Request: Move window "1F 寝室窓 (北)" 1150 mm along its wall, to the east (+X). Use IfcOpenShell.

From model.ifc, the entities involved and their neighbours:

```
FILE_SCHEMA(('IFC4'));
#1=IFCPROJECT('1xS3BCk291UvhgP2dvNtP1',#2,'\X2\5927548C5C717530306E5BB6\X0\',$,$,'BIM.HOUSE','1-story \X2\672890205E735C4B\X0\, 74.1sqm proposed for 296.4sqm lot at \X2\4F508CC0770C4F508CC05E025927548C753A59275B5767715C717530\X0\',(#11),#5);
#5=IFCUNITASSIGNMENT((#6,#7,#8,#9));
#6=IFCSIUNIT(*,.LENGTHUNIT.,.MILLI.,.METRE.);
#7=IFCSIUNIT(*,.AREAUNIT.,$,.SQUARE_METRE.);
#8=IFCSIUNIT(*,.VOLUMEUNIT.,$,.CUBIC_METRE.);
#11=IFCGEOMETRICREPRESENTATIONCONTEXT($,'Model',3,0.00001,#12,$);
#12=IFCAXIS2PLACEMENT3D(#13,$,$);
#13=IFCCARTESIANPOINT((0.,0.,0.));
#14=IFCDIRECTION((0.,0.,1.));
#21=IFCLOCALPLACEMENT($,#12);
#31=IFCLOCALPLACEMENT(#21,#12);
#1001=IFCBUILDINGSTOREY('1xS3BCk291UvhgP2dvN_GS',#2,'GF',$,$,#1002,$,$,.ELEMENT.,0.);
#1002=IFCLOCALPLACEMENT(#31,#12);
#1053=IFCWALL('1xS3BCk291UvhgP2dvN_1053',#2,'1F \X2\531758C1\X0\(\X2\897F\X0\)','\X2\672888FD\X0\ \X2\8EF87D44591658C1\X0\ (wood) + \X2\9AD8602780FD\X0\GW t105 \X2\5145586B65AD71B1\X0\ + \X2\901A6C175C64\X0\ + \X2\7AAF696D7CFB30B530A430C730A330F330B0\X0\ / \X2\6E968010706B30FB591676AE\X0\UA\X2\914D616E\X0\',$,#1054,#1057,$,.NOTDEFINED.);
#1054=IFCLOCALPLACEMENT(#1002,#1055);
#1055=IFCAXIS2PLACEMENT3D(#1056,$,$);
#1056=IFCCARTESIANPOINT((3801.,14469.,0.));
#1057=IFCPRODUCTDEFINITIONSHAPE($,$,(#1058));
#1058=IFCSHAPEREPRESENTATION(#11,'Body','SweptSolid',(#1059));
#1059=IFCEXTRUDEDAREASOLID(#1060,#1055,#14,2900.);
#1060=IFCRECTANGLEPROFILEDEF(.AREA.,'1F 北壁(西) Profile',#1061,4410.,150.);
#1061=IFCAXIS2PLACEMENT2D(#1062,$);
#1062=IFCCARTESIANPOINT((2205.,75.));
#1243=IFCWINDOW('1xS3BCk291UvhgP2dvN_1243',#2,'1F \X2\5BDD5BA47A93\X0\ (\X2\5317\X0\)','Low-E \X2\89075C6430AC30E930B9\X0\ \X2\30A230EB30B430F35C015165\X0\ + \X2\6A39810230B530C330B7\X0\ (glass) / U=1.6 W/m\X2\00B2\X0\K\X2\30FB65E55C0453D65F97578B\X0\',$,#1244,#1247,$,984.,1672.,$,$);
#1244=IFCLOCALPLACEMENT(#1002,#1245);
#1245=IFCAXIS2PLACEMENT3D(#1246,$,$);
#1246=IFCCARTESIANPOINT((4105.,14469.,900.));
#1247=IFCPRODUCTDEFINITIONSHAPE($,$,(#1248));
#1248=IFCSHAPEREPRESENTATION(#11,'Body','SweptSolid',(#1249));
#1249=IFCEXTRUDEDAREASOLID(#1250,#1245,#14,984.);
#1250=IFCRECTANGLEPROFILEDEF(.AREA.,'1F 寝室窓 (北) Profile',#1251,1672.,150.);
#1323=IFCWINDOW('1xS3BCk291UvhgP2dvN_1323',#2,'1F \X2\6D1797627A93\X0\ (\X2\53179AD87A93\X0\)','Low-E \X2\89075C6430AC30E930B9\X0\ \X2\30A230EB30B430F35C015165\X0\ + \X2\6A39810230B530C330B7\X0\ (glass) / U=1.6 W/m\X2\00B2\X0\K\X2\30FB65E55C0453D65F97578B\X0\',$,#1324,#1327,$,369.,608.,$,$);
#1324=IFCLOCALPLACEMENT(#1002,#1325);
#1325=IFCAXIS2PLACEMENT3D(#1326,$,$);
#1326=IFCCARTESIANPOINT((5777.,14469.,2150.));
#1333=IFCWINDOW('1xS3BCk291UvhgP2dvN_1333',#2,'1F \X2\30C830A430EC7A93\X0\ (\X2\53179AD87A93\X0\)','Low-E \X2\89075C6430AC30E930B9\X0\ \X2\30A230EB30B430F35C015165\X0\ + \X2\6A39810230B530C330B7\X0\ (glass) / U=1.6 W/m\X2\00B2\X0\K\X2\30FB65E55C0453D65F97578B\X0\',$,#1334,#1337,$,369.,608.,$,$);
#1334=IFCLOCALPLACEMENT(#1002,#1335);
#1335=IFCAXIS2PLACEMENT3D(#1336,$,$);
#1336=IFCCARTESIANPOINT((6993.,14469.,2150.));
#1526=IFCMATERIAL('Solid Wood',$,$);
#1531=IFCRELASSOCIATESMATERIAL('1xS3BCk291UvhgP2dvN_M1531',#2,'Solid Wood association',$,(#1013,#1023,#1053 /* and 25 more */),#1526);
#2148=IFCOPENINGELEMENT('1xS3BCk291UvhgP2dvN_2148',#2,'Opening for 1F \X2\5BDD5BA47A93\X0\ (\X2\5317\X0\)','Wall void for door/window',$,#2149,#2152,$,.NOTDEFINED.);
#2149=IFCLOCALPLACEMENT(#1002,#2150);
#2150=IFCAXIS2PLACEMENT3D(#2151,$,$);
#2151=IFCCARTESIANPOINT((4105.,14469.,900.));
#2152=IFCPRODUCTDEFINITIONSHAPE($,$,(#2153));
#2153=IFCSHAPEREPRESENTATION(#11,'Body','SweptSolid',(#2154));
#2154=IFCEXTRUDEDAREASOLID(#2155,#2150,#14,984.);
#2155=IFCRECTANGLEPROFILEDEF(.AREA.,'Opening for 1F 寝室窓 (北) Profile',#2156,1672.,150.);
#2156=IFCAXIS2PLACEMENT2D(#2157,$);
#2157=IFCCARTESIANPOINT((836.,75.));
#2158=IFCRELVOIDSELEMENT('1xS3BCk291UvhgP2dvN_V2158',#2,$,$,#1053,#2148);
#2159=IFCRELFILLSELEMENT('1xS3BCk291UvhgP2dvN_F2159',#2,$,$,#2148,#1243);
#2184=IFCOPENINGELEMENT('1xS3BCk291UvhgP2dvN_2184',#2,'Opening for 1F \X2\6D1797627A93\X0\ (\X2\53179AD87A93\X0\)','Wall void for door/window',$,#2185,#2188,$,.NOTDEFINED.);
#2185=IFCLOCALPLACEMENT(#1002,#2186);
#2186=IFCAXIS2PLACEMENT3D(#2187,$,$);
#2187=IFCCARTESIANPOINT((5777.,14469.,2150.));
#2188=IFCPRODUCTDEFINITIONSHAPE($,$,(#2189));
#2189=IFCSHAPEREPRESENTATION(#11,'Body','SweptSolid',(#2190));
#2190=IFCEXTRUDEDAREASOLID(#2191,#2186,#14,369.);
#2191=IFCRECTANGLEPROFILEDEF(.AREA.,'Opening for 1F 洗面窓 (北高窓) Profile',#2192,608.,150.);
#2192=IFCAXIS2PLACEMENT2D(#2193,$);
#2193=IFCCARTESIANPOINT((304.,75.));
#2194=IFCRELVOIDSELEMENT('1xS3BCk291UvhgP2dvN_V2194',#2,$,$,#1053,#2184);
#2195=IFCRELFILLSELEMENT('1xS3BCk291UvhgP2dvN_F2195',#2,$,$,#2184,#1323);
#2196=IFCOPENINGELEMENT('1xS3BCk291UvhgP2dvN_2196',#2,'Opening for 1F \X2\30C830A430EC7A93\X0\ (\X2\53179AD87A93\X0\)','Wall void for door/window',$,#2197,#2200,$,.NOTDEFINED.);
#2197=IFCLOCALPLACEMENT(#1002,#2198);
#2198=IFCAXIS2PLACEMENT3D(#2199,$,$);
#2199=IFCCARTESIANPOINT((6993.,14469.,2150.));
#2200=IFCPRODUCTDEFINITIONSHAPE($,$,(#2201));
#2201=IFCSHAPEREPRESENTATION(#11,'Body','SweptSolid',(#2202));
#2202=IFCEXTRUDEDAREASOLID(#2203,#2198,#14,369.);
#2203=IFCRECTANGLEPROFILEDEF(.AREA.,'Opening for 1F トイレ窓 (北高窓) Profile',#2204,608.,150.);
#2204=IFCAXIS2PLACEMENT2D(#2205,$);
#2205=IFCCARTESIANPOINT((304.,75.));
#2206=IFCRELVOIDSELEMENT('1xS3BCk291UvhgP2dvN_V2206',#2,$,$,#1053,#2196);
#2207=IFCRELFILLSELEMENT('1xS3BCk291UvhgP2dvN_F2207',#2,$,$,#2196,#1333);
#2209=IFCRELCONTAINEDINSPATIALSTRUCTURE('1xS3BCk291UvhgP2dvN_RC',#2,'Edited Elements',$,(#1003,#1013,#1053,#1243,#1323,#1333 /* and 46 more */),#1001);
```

```python
import ifcopenshell
import ifcopenshell.api.geometry
import ifcopenshell.util.placement
import ifcopenshell.util.unit

model = ifcopenshell.open("model.ifc")
unit_scale = ifcopenshell.util.unit.calculate_unit_scale(model)

window = model.by_guid("1xS3BCk291UvhgP2dvN_1243")
opening = window.FillsVoids[0].RelatingOpeningElement
wall = opening.VoidsElements[0].RelatingBuildingElement

wall_matrix = ifcopenshell.util.placement.get_local_placement(wall.ObjectPlacement)
shift = wall_matrix[:3, 0] * 1.15 / unit_scale
before = ifcopenshell.util.placement.get_local_placement(window.ObjectPlacement)[:3, 3].copy()

# The window is not placed relative to its opening, so move both.
for product in (opening, window):
    matrix = ifcopenshell.util.placement.get_local_placement(product.ObjectPlacement)
    matrix[:3, 3] += shift
    ifcopenshell.api.geometry.edit_object_placement(model, product=product, matrix=matrix, is_si=False)

after = ifcopenshell.util.placement.get_local_placement(window.ObjectPlacement)[:3, 3]
print("window moved by", (after - before).round(3) + 0.0)

model.write("model_edited.ifc")
```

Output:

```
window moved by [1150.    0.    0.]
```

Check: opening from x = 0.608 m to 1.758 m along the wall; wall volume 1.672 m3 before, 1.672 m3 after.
